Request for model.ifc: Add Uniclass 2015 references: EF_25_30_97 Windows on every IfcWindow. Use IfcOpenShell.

First a look at what the model holds.

```python
import ifcopenshell

model = ifcopenshell.open("model.ifc")
print(model.schema)
print("classifications:", [c.Name for c in model.by_type("IfcClassification")])
for ifc_class in ("IfcDoor", "IfcRoof", "IfcStair", "IfcWall", "IfcWindow"):
    print(ifc_class, len(model.by_type(ifc_class)))
```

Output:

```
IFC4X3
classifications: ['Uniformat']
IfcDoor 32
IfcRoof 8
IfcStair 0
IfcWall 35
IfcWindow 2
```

```python
import ifcopenshell
import ifcopenshell.api.classification

model = ifcopenshell.open("model.ifc")

system = ifcopenshell.api.classification.add_classification(model, classification="Uniclass 2015")

codes = {
    "IfcWindow": ("EF_25_30_97", "Windows"),
}
for ifc_class, (code, name) in codes.items():
    products = model.by_type(ifc_class)
    ifcopenshell.api.classification.add_reference(
        model, products=products, classification=system, identification=code, name=name
    )
    print(code, len(products))

model.write("model_updated.ifc")
```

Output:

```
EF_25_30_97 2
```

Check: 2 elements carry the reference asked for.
